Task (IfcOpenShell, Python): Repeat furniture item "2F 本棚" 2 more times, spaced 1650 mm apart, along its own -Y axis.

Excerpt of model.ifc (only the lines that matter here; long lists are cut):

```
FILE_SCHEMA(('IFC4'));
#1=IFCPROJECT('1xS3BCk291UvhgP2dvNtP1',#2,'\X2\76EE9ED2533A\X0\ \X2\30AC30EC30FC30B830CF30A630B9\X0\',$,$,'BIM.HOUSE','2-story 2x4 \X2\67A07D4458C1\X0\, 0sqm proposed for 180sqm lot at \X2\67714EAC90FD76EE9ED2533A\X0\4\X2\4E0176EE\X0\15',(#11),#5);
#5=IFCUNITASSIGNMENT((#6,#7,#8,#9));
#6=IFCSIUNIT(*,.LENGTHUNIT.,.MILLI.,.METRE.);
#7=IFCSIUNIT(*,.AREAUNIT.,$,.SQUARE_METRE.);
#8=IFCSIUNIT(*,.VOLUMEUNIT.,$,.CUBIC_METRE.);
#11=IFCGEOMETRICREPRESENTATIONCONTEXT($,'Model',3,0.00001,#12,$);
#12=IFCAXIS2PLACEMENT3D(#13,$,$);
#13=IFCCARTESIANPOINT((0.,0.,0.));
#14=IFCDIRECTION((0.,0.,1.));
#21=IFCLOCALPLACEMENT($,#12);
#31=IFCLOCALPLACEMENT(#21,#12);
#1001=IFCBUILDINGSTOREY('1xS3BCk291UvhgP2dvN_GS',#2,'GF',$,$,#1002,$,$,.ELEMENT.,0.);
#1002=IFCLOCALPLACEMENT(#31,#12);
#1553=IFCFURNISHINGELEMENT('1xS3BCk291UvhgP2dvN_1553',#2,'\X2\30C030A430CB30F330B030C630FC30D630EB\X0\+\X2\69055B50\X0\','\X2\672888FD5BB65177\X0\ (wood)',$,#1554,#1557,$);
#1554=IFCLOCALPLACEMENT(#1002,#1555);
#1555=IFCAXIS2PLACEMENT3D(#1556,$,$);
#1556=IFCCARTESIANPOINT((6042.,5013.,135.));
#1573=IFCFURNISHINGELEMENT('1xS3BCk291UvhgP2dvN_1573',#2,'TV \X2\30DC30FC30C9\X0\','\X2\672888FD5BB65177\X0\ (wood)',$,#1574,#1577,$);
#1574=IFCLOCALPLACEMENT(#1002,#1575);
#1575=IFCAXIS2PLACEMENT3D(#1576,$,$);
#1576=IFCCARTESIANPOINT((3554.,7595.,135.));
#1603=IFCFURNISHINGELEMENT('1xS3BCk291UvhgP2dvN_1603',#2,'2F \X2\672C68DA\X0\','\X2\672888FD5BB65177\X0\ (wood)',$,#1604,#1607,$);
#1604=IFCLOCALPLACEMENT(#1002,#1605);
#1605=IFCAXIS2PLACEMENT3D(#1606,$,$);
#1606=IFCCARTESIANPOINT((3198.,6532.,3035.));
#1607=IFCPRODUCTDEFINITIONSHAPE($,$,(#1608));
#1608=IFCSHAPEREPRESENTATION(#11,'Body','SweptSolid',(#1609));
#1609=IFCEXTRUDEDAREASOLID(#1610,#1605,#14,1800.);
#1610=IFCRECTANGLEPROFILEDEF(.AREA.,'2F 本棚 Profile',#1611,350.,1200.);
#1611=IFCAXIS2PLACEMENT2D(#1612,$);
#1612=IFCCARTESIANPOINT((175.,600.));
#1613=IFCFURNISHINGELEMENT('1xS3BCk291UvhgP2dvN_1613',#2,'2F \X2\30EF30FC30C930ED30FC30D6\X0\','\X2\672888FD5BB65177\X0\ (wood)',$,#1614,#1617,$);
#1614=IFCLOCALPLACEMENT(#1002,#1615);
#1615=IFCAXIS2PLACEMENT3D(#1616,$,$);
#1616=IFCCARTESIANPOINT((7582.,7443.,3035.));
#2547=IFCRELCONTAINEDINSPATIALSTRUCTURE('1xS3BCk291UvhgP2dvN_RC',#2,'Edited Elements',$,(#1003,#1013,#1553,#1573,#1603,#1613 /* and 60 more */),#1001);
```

```python
import ifcopenshell
import ifcopenshell.api.geometry
import ifcopenshell.api.root
import ifcopenshell.util.element
import ifcopenshell.util.placement

model = ifcopenshell.open("model.ifc")


def reuse_history(source, copy):
    """copy_class also copies each property set's owner history, people and application; keep the originals."""
    for rel in copy.IsDefinedBy:
        if rel.is_a("IfcRelDefinesByProperties") and (history := rel.RelatingPropertyDefinition.OwnerHistory):
            rel.RelatingPropertyDefinition.OwnerHistory = source.OwnerHistory
            ifcopenshell.util.element.remove_deep2(model, history)


source = model.by_guid("1xS3BCk291UvhgP2dvN_1603")
base = ifcopenshell.util.placement.get_local_placement(source.ObjectPlacement)
step = -base[:3, 1] * 1650.0

for i in range(1, 3):
    copy = ifcopenshell.api.root.copy_class(model, product=source)
    copy.Representation = ifcopenshell.util.element.copy_deep(
        model, source.Representation, exclude=["IfcGeometricRepresentationContext", "IfcRepresentationMap"]
    )
    reuse_history(source, copy)
    matrix = base.copy()
    matrix[:3, 3] += i * step
    print("added at", matrix[:3, 3].round(3) + 0.0)
    ifcopenshell.api.geometry.edit_object_placement(model, product=copy, matrix=matrix, is_si=False)

model.write("model_v2.ifc")
```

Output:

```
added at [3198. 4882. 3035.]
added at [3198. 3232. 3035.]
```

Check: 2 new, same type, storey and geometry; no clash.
